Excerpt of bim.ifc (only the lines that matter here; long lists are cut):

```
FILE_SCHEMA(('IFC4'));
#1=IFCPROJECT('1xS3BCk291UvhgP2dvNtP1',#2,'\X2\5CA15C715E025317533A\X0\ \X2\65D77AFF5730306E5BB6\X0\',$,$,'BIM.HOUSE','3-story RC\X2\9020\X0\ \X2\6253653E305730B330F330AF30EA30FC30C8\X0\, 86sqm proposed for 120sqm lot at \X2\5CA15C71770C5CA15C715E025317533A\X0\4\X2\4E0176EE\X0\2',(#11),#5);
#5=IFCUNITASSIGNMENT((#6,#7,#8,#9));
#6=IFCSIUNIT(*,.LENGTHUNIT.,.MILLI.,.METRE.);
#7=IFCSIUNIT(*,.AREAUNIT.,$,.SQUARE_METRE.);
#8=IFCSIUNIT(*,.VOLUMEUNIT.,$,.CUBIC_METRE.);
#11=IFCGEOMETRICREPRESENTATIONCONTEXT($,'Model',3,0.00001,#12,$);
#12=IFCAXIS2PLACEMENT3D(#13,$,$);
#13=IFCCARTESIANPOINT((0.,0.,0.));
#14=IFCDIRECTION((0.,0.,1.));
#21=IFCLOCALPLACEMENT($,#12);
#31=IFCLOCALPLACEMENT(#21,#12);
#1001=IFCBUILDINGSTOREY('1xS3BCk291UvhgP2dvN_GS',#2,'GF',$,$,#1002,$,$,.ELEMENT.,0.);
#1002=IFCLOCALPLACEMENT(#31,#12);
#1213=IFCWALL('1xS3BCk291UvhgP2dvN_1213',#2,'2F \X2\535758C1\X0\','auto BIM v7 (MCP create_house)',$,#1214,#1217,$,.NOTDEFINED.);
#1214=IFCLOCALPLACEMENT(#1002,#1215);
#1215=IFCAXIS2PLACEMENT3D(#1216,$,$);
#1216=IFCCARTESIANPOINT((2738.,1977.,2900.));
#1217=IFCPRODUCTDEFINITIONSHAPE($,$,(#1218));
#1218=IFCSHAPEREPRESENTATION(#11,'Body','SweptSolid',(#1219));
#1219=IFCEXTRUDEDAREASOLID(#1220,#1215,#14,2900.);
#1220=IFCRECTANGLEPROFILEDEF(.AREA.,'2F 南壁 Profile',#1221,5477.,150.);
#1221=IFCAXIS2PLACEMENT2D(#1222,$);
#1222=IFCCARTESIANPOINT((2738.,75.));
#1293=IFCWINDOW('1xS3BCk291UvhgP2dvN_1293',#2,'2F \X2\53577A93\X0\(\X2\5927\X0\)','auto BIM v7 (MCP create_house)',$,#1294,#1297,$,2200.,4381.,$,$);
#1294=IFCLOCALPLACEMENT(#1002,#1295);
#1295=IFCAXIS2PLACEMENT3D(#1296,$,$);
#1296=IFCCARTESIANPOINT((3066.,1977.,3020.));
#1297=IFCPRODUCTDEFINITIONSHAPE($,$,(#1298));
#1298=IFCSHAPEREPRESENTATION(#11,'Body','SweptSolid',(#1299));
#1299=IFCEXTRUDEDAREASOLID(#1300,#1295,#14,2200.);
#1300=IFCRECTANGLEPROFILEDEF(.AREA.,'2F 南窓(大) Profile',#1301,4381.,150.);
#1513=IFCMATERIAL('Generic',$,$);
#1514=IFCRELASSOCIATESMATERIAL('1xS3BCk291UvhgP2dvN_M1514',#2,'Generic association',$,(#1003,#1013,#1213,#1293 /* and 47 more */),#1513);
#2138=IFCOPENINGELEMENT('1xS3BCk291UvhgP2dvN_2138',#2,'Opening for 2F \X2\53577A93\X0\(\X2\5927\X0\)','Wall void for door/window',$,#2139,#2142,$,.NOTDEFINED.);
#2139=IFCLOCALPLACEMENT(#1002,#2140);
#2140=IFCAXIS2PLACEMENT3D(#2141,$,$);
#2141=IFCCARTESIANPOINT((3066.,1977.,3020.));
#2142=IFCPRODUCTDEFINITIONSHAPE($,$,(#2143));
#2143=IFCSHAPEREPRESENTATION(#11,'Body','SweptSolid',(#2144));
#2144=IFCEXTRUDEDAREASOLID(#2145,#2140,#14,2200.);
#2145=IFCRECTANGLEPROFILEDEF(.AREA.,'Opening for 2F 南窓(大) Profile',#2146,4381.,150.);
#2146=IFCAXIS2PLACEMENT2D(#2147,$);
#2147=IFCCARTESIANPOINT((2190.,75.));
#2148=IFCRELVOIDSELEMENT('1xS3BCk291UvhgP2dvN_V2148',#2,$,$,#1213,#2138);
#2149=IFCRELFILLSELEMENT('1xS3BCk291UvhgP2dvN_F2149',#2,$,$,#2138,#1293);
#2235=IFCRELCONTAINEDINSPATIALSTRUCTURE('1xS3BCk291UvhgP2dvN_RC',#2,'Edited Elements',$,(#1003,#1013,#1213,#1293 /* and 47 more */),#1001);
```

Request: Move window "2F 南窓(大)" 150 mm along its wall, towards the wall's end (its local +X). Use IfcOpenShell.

```python
import ifcopenshell
import ifcopenshell.api.geometry
import ifcopenshell.util.placement

model = ifcopenshell.open("bim.ifc")

window = model.by_guid("1xS3BCk291UvhgP2dvN_1293")
opening = window.FillsVoids[0].RelatingOpeningElement
wall = opening.VoidsElements[0].RelatingBuildingElement

wall_matrix = ifcopenshell.util.placement.get_local_placement(wall.ObjectPlacement)
shift = wall_matrix[:3, 0] * 150.0
before = ifcopenshell.util.placement.get_local_placement(window.ObjectPlacement)[:3, 3].copy()

# The window is not placed relative to its opening, so move both.
for product in (opening, window):
    matrix = ifcopenshell.util.placement.get_local_placement(product.ObjectPlacement)
    matrix[:3, 3] += shift
    ifcopenshell.api.geometry.edit_object_placement(model, product=product, matrix=matrix, is_si=False)

after = ifcopenshell.util.placement.get_local_placement(window.ObjectPlacement)[:3, 3]
print("window moved by", (after - before).round(3) + 0.0)

model.write("bim-out.ifc")
```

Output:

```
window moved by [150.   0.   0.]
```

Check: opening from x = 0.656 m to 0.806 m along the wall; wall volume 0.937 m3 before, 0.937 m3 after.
